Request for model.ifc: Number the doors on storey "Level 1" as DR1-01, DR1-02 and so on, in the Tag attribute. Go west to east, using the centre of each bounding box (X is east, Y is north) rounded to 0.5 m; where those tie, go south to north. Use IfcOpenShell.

First a look at what the model holds.

```python
import ifcopenshell
import ifcopenshell.util.element
import ifcopenshell.util.placement

model = ifcopenshell.open("model.ifc")
print(model.schema)
storey = next(s for s in model.by_type("IfcBuildingStorey") if s.Name == "Level 1")
doors = [e for e in ifcopenshell.util.element.get_decomposition(storey) if e.is_a("IfcDoor")]
for e in sorted(doors, key=lambda e: e.id()):
    origin = ifcopenshell.util.placement.get_local_placement(e.ObjectPlacement)[:3, 3]
    print(e.id(), e.Tag, e.Name, origin.round(2) + 0.0, sep=" | ")
```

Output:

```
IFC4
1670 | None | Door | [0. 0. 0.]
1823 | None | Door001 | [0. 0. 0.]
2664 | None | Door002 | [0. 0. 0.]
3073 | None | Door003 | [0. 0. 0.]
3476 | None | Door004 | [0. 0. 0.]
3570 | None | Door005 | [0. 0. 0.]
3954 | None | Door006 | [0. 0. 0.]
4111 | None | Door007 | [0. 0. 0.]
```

```python
import ifcopenshell
import ifcopenshell.geom
import ifcopenshell.util.element
import ifcopenshell.util.shape

model = ifcopenshell.open("model.ifc")
settings = ifcopenshell.geom.settings()
settings.set("use-world-coords", True)


def centre(element):
    shape = ifcopenshell.geom.create_shape(settings, element)
    return ifcopenshell.util.shape.get_bbox_centroid(shape.geometry)


storey = next(s for s in model.by_type("IfcBuildingStorey") if s.Name == "Level 1")
doors = [e for e in ifcopenshell.util.element.get_decomposition(storey) if e.is_a("IfcDoor")]

# Insertion points can sit at a corner or the storey origin, so sort by the geometry (in metres).
centres = {e: centre(e) for e in doors}
doors.sort(key=lambda e: (round(centres[e][0] / 0.5), centres[e][1]))

for i, e in enumerate(doors, start=1):
    number = f"DR1-{i:02d}"
    e.Tag = number
    print(e.id(), number)

model.write("model-out.ifc")
```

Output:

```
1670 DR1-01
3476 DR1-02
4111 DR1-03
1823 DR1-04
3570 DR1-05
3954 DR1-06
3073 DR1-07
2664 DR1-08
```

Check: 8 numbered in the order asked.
